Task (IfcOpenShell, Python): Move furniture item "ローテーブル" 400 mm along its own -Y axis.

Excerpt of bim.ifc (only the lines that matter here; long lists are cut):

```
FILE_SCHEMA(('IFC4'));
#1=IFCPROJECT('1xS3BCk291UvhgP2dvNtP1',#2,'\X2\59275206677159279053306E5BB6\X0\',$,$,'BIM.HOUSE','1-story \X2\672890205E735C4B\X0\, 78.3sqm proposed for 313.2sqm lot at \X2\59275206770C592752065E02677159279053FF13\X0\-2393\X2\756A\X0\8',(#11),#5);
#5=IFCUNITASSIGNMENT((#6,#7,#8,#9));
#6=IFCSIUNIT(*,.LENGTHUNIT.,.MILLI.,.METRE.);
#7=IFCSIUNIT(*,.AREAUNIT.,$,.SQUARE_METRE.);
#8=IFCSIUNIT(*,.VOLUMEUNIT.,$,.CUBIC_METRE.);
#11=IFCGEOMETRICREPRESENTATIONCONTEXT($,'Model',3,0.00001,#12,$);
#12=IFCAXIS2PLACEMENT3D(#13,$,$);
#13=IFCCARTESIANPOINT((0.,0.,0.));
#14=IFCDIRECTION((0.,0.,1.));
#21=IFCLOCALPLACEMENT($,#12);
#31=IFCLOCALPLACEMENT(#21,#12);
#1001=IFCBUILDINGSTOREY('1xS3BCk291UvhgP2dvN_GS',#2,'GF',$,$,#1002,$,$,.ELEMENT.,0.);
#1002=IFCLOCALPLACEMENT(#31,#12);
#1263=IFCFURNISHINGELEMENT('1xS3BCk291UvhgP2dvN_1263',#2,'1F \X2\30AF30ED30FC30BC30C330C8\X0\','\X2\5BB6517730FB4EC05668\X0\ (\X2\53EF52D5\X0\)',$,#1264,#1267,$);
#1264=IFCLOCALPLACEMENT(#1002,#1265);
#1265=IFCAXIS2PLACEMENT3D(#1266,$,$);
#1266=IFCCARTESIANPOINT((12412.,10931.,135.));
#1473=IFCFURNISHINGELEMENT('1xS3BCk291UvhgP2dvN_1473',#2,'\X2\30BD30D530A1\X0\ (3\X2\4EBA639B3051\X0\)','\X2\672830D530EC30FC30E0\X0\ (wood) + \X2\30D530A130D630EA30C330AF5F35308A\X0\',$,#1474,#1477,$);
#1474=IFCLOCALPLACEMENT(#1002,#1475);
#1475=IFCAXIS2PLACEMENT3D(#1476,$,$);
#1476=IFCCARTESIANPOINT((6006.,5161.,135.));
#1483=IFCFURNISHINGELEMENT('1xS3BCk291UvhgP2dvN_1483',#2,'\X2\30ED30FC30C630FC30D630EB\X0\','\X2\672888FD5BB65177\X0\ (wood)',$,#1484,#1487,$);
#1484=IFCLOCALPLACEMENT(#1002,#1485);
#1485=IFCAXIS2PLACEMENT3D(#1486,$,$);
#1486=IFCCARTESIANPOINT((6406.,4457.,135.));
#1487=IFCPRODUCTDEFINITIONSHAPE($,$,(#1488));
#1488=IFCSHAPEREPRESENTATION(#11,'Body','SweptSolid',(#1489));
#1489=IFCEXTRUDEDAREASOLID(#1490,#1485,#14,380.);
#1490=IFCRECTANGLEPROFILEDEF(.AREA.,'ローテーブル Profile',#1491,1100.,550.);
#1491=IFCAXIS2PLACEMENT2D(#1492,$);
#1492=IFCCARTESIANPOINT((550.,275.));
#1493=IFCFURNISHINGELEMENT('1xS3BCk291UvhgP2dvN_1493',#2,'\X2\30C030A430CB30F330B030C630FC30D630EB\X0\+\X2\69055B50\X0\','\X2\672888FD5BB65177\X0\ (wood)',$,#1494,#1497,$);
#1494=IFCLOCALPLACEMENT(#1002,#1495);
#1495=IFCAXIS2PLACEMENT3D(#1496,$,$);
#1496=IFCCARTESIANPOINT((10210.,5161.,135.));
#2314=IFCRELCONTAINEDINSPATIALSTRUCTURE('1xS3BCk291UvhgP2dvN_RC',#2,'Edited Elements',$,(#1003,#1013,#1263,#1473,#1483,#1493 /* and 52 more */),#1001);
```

```python
import ifcopenshell
import ifcopenshell.api.geometry
import ifcopenshell.util.placement

model = ifcopenshell.open("bim.ifc")

item = model.by_guid("1xS3BCk291UvhgP2dvN_1483")
matrix = ifcopenshell.util.placement.get_local_placement(item.ObjectPlacement)
matrix[:3, 3] -= matrix[:3, 1] * 400.0
ifcopenshell.api.geometry.edit_object_placement(model, product=item, matrix=matrix, is_si=False)

print(ifcopenshell.util.placement.get_local_placement(item.ObjectPlacement).round(3) + 0.0)

model.write("bim_updated.ifc")
```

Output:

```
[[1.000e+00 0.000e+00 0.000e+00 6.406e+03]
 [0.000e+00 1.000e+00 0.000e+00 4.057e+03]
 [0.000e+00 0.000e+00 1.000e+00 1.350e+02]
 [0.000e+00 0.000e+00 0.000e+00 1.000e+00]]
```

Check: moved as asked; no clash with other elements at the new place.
